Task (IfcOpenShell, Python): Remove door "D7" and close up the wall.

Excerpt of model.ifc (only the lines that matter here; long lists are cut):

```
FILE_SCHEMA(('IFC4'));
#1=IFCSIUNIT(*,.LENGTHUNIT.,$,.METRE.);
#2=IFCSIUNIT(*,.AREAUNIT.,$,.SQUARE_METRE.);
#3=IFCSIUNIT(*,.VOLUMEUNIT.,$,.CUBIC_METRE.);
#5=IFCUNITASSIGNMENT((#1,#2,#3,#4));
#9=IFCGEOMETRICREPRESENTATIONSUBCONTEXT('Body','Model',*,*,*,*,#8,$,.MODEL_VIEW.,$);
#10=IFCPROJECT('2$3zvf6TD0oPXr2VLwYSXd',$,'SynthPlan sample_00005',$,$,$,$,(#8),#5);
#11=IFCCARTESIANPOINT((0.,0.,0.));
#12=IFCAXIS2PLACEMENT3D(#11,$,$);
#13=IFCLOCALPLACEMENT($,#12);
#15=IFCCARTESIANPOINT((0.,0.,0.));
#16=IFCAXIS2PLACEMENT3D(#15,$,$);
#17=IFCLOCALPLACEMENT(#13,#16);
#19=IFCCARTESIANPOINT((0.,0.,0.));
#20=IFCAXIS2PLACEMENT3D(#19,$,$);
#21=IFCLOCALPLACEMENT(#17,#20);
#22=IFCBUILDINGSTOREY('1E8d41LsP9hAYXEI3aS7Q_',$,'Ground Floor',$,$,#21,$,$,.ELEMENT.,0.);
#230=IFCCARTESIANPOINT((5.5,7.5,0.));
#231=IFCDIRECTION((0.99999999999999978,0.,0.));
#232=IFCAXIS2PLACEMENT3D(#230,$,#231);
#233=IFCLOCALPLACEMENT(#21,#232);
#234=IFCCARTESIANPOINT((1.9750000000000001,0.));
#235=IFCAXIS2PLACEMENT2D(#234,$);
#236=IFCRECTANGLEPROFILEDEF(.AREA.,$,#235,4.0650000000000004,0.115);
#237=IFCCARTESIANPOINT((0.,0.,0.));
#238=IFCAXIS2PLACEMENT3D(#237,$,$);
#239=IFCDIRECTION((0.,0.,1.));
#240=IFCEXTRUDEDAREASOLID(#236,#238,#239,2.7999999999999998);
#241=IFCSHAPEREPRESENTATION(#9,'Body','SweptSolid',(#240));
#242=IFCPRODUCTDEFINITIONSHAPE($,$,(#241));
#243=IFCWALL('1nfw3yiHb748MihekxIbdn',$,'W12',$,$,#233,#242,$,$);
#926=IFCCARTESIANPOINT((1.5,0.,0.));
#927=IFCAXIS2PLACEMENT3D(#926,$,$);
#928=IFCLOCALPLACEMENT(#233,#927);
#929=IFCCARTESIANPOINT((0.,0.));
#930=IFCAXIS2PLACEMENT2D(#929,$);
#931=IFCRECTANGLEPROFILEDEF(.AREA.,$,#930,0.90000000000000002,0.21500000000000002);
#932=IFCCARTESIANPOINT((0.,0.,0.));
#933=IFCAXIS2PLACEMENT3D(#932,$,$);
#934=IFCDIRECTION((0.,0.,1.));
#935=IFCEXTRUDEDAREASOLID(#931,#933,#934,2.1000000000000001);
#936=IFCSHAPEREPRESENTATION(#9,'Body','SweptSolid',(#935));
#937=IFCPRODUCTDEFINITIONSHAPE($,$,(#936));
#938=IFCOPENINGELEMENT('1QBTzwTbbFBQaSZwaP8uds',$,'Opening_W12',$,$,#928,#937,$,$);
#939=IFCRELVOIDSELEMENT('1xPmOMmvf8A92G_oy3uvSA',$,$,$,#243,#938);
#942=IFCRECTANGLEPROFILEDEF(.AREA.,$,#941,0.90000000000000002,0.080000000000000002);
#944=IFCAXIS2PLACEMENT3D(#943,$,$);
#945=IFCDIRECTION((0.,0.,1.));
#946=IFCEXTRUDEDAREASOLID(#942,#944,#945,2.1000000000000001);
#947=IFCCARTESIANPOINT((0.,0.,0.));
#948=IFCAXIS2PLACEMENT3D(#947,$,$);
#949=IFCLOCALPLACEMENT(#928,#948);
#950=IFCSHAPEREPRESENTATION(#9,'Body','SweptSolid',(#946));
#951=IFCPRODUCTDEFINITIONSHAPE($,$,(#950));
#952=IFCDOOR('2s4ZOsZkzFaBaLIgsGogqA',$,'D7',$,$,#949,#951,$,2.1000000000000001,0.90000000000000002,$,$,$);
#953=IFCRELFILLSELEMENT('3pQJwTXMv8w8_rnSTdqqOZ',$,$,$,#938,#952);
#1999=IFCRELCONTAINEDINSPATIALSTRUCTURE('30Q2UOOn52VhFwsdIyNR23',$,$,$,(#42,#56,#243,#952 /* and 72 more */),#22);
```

```python
import ifcopenshell
import ifcopenshell.api.feature
import ifcopenshell.api.root
import ifcopenshell.geom
import ifcopenshell.util.shape

model = ifcopenshell.open("model.ifc")
settings = ifcopenshell.geom.settings()


def volume(element):
    """Net volume in cubic metres, openings subtracted."""
    shape = ifcopenshell.geom.create_shape(settings, element)
    return ifcopenshell.util.shape.get_volume(shape.geometry)


door = model.by_guid("2s4ZOsZkzFaBaLIgsGogqA")
opening = door.FillsVoids[0].RelatingOpeningElement
wall = opening.VoidsElements[0].RelatingBuildingElement
before = volume(wall)

ifcopenshell.api.root.remove_product(model, product=door)
ifcopenshell.api.feature.remove_feature(model, feature=opening)

after = volume(wall)

print(f"wall volume {before:.3f} -> {after:.3f} m3")

model.write("model_rev.ifc")
```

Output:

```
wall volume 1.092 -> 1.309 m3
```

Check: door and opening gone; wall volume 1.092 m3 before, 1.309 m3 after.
